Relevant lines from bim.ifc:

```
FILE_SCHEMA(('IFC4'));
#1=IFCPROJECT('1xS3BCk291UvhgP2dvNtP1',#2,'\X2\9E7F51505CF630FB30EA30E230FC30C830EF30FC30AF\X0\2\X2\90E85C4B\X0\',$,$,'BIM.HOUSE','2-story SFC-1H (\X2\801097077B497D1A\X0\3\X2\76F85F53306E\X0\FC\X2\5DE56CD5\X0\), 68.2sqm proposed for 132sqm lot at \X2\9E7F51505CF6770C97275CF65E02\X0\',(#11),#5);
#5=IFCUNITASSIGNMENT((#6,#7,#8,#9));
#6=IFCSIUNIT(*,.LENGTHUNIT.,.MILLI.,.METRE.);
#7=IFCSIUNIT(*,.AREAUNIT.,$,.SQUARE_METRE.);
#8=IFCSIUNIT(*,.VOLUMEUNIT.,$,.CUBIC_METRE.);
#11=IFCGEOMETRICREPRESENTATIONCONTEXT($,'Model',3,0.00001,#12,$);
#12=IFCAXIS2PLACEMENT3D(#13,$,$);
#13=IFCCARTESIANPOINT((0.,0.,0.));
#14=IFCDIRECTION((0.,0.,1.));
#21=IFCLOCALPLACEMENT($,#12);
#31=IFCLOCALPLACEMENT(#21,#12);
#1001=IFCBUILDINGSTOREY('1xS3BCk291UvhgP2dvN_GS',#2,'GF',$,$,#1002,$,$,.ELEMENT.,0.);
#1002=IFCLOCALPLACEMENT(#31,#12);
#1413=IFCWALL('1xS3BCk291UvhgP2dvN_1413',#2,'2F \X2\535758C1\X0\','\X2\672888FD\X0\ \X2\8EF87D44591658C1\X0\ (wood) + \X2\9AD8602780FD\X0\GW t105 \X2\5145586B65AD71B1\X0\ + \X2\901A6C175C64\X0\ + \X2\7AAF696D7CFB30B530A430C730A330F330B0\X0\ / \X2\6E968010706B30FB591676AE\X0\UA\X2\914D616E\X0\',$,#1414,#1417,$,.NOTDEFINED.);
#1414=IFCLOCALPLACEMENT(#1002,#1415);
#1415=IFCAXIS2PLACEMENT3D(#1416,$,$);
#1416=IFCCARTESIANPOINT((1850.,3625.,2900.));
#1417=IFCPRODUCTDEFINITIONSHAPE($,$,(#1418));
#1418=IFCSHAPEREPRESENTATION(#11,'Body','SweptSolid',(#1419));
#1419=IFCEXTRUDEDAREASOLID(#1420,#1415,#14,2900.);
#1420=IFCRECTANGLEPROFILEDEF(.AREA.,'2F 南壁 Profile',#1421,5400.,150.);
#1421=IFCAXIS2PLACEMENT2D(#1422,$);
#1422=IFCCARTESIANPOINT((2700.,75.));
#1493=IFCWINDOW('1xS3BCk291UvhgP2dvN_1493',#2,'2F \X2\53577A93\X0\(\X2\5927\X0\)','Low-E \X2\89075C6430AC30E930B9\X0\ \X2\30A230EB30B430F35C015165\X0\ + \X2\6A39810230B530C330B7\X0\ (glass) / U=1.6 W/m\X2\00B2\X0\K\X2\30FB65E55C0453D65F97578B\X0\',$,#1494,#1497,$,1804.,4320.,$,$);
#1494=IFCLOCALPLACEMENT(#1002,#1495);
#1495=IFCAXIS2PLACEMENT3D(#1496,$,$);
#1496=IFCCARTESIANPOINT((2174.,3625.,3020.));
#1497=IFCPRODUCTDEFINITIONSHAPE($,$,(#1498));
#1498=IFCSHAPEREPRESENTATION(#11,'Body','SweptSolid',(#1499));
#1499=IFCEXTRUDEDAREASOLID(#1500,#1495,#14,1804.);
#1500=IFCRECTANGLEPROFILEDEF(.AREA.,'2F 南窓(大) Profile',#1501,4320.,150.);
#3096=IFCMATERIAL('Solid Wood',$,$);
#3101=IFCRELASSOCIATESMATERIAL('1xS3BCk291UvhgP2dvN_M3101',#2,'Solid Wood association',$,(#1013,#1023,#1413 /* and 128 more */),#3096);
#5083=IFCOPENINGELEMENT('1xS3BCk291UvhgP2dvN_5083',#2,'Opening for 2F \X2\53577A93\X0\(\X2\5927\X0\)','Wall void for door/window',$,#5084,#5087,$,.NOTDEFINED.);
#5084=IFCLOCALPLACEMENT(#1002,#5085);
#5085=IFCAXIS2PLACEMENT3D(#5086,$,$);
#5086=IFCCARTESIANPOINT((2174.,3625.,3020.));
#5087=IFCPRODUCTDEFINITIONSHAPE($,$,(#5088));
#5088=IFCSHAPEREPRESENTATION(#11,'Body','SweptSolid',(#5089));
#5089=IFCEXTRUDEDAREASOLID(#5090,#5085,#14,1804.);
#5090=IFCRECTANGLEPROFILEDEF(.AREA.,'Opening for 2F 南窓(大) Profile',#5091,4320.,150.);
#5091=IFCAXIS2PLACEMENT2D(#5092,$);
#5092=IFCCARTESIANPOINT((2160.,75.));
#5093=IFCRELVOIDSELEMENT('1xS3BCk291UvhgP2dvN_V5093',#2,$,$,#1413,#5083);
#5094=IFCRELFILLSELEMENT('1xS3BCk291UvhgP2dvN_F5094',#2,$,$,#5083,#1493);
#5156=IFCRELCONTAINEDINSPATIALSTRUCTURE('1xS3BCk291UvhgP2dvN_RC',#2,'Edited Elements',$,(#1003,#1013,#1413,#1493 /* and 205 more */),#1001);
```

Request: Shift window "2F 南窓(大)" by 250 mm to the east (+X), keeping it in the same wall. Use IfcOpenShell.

```python
import ifcopenshell
import ifcopenshell.api.geometry
import ifcopenshell.util.placement

model = ifcopenshell.open("bim.ifc")

window = model.by_id(1493)
opening = window.FillsVoids[0].RelatingOpeningElement
wall = opening.VoidsElements[0].RelatingBuildingElement

wall_matrix = ifcopenshell.util.placement.get_local_placement(wall.ObjectPlacement)
shift = wall_matrix[:3, 0] * 250.0
before = ifcopenshell.util.placement.get_local_placement(window.ObjectPlacement)[:3, 3].copy()

# The window is not placed relative to its opening, so move both.
for product in (opening, window):
    matrix = ifcopenshell.util.placement.get_local_placement(product.ObjectPlacement)
    matrix[:3, 3] += shift
    ifcopenshell.api.geometry.edit_object_placement(model, product=product, matrix=matrix, is_si=False)

after = ifcopenshell.util.placement.get_local_placement(window.ObjectPlacement)[:3, 3]
print("window moved by", (after - before).round(3) + 0.0)

model.write("bim-out.ifc")
```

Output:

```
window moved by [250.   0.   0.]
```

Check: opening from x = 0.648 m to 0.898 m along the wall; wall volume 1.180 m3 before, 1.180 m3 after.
